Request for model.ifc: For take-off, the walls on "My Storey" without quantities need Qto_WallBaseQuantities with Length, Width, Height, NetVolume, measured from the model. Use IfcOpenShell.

First a look at what the model holds.

```python
import ifcopenshell
import ifcopenshell.util.element
import ifcopenshell.util.unit

model = ifcopenshell.open("model.ifc")
print(model.schema)
for unit_type in ("LENGTHUNIT", "AREAUNIT", "VOLUMEUNIT"):
    print(unit_type, ifcopenshell.util.unit.calculate_unit_scale(model, unit_type))
storey = next(s for s in model.by_type("IfcBuildingStorey") if s.Name == "My Storey")
walls = [e for e in ifcopenshell.util.element.get_decomposition(storey) if e.is_a("IfcWall")]
for e in sorted(walls, key=lambda e: e.id()):
    print(e.id(), e.is_a(), e.Name, list(ifcopenshell.util.element.get_psets(e, qtos_only=True)), sep=" | ")
```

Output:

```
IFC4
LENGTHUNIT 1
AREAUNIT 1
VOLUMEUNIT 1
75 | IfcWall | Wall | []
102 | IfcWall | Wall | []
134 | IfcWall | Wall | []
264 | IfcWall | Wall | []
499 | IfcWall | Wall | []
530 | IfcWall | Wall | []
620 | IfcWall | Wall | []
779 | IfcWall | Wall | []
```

```python
import ifcopenshell
import ifcopenshell.api.pset
import ifcopenshell.geom
import ifcopenshell.util.element
import ifcopenshell.util.shape
import ifcopenshell.util.unit

model = ifcopenshell.open("model.ifc")
unit_scale = ifcopenshell.util.unit.calculate_unit_scale(model)
volume_scale = ifcopenshell.util.unit.calculate_unit_scale(model, "VOLUMEUNIT")
settings = ifcopenshell.geom.settings()

storey = next(s for s in model.by_type("IfcBuildingStorey") if s.Name == "My Storey")
walls = [e for e in ifcopenshell.util.element.get_decomposition(storey) if e.is_a("IfcWall")]

for e in sorted(walls, key=lambda e: e.id()):
    if ifcopenshell.util.element.get_psets(e, qtos_only=True, should_inherit=False):
        continue
    # Geometry comes back in metres, in the element's own axes.
    shape = ifcopenshell.geom.create_shape(settings, e)
    values = {
        "Length": ifcopenshell.util.shape.get_x(shape.geometry) / unit_scale,
        "Width": ifcopenshell.util.shape.get_y(shape.geometry) / unit_scale,
        "Height": ifcopenshell.util.shape.get_z(shape.geometry) / unit_scale,
        "NetVolume": ifcopenshell.util.shape.get_volume(shape.geometry) / volume_scale,
    }
    qto = ifcopenshell.api.pset.add_qto(model, product=e, name="Qto_WallBaseQuantities")
    ifcopenshell.api.pset.edit_qto(model, qto=qto, properties=values)
    print(e.id(), {k: round(v, 3) for k, v in values.items()})

model.write("model_v2.ifc")
```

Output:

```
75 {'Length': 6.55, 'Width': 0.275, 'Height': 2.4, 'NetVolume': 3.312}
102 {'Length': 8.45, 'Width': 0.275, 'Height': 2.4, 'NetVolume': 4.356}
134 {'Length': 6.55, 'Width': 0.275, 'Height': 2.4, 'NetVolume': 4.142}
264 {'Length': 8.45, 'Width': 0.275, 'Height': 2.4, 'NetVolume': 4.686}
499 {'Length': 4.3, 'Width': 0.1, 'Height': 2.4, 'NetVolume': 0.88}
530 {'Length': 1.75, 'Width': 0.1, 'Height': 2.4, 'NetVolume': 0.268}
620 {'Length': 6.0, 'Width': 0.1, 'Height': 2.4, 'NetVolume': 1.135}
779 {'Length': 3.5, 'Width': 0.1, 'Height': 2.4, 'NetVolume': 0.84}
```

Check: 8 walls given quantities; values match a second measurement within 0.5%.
